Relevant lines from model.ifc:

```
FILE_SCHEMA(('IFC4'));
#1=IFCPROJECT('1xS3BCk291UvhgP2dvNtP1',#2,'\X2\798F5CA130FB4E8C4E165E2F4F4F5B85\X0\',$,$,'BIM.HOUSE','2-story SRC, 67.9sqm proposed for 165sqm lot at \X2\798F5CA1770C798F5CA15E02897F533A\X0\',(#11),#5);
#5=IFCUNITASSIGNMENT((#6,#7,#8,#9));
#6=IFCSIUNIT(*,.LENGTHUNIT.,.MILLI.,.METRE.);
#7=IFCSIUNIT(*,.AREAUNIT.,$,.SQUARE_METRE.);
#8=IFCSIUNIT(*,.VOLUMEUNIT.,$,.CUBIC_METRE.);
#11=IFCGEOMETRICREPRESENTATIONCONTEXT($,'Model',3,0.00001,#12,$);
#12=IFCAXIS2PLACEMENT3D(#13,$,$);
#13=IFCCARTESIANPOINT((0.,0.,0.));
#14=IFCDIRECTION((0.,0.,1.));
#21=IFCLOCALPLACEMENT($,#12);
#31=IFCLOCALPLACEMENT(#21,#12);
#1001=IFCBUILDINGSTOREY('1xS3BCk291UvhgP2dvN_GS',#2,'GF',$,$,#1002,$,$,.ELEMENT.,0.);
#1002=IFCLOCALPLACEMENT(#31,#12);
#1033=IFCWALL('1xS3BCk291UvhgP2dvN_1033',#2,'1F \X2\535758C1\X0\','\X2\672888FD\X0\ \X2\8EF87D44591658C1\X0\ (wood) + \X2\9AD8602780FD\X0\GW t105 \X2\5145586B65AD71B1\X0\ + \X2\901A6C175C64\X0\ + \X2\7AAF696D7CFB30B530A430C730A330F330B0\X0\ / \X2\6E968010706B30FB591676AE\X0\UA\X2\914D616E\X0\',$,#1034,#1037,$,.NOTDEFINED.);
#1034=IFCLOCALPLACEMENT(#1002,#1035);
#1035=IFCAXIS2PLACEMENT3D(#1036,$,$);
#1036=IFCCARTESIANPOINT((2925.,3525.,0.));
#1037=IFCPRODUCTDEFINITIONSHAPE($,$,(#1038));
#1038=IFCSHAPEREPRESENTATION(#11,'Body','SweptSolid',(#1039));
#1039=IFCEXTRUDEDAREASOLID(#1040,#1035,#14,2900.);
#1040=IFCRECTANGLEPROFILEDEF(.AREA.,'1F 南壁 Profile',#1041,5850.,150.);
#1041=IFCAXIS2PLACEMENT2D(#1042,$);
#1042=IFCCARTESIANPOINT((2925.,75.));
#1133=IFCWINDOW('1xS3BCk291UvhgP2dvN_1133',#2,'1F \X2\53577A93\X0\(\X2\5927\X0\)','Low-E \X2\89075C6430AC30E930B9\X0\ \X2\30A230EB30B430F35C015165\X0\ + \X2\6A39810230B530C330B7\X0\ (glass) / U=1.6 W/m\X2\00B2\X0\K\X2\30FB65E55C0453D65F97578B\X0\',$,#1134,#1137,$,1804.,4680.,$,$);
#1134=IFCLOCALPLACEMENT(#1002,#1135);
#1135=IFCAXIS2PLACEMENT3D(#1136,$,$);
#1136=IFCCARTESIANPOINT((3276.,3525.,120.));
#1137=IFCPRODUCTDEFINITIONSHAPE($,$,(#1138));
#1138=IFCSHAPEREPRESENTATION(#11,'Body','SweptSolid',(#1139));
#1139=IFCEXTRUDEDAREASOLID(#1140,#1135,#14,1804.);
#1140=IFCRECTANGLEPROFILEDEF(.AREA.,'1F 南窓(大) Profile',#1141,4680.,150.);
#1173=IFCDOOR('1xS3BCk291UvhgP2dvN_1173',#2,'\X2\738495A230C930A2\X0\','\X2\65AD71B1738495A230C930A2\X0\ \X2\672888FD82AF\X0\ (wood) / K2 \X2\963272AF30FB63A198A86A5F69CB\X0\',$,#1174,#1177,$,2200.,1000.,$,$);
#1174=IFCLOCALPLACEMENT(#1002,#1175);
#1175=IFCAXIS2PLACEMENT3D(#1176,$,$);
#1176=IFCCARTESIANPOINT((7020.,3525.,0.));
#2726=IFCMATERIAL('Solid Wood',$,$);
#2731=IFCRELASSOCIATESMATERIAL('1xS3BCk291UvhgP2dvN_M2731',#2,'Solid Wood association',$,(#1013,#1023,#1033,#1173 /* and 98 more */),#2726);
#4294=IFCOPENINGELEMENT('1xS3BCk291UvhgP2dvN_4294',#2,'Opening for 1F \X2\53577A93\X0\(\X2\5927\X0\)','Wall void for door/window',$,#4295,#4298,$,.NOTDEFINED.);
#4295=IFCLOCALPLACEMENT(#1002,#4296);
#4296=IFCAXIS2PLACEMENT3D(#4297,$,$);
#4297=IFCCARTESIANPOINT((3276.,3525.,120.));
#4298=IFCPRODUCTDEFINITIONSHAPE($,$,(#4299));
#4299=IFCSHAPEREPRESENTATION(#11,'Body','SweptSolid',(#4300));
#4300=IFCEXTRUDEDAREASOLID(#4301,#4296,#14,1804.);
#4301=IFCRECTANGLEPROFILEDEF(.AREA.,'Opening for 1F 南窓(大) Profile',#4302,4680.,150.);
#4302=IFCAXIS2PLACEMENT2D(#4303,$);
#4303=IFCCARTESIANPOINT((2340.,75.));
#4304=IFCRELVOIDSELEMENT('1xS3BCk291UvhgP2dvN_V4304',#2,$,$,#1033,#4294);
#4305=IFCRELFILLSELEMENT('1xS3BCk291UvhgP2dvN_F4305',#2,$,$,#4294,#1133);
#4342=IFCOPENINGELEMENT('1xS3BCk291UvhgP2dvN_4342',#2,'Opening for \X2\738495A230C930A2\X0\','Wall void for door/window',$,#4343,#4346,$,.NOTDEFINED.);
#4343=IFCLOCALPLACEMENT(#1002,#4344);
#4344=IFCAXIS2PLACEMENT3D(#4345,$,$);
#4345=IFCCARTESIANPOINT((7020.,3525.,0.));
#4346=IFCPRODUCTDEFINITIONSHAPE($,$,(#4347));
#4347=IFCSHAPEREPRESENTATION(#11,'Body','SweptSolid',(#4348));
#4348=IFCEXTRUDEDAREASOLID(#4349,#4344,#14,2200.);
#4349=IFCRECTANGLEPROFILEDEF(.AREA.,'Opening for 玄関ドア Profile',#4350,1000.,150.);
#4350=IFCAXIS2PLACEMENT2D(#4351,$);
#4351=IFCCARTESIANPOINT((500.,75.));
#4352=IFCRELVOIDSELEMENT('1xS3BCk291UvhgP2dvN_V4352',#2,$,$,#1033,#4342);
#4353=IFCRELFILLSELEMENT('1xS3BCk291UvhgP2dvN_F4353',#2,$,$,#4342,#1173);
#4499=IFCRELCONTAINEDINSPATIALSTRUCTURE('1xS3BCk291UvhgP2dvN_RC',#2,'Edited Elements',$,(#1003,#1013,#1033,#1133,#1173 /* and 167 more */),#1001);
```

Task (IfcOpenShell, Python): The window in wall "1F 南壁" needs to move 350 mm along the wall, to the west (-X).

```python
import ifcopenshell
import ifcopenshell.api.geometry
import ifcopenshell.util.placement

model = ifcopenshell.open("model.ifc")

window = model.by_guid("1xS3BCk291UvhgP2dvN_1133")
opening = window.FillsVoids[0].RelatingOpeningElement
wall = opening.VoidsElements[0].RelatingBuildingElement

wall_matrix = ifcopenshell.util.placement.get_local_placement(wall.ObjectPlacement)
shift = wall_matrix[:3, 0] * -350.0
before = ifcopenshell.util.placement.get_local_placement(window.ObjectPlacement)[:3, 3].copy()

# The window is not placed relative to its opening, so move both.
for product in (opening, window):
    matrix = ifcopenshell.util.placement.get_local_placement(product.ObjectPlacement)
    matrix[:3, 3] += shift
    ifcopenshell.api.geometry.edit_object_placement(model, product=product, matrix=matrix, is_si=False)

after = ifcopenshell.util.placement.get_local_placement(window.ObjectPlacement)[:3, 3]
print("window moved by", (after - before).round(3) + 0.0)

model.write("model_rev.ifc")
```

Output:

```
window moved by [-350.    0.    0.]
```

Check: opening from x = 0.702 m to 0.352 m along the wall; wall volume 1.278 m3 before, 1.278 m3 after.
